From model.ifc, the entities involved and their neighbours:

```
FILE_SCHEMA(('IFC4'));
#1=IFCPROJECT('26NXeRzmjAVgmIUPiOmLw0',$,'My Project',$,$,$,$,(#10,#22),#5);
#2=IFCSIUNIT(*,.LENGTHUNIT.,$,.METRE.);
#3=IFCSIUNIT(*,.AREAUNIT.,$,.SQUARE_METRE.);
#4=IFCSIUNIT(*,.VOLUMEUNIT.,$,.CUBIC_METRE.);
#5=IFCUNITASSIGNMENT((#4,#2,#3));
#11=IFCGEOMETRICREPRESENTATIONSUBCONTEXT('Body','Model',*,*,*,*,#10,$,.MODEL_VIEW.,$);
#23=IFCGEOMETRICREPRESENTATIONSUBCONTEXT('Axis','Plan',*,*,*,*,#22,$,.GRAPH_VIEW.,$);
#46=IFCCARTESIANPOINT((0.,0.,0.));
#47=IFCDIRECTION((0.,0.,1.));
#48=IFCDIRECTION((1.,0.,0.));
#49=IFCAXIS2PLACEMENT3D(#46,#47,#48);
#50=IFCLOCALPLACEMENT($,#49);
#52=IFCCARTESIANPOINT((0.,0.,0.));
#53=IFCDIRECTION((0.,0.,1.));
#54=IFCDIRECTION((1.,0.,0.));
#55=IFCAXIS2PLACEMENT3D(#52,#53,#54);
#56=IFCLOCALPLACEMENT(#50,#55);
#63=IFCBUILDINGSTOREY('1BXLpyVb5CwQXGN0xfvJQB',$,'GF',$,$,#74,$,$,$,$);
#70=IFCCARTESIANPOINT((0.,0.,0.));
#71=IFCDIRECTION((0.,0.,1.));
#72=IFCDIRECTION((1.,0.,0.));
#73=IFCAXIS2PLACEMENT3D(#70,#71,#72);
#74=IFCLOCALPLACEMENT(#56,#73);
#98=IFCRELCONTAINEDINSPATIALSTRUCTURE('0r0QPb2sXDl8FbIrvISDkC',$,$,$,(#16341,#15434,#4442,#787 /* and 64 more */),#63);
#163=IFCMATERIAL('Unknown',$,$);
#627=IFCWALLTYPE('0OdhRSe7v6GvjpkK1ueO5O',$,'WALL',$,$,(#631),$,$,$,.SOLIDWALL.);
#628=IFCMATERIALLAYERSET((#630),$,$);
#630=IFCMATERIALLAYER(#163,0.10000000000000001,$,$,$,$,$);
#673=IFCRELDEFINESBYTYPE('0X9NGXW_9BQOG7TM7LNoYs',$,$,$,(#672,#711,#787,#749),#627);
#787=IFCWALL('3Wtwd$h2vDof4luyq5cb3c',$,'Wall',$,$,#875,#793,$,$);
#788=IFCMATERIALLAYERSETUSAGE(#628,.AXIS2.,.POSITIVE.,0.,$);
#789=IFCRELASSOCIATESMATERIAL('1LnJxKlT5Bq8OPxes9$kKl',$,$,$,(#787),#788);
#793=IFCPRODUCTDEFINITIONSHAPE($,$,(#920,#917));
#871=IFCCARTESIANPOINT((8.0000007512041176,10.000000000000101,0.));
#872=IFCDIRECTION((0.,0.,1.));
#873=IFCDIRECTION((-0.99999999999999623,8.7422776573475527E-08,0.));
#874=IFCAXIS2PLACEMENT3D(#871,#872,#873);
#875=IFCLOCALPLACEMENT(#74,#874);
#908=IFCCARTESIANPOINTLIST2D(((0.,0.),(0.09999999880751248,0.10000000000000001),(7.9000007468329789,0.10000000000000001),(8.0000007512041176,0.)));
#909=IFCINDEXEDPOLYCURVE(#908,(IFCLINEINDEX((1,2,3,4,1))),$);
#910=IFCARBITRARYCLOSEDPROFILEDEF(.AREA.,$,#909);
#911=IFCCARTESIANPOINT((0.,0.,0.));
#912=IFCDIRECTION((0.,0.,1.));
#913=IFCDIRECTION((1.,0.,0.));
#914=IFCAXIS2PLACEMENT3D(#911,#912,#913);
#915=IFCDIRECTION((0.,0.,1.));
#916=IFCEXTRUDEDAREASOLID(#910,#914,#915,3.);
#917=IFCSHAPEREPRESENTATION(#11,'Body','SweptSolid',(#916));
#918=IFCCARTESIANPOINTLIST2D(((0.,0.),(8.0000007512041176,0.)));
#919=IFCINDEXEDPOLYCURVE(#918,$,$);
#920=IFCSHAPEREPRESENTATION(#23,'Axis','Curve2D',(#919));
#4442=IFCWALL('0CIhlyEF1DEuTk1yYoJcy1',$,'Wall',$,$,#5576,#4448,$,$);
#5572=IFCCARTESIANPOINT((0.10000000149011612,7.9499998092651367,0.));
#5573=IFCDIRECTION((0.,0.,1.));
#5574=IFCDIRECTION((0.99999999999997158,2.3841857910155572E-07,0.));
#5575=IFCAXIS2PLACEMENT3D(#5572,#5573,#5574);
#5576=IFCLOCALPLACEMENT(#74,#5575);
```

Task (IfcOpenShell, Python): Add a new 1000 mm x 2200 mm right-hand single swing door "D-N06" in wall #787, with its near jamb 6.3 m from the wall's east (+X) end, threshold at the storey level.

```python
import numpy as np
import ifcopenshell
import ifcopenshell.api.feature
import ifcopenshell.api.geometry
import ifcopenshell.api.root
import ifcopenshell.api.spatial
import ifcopenshell.geom
import ifcopenshell.util.element
import ifcopenshell.util.placement
import ifcopenshell.util.representation
import ifcopenshell.util.shape
import ifcopenshell.util.unit

model = ifcopenshell.open("model.ifc")
unit_scale = ifcopenshell.util.unit.calculate_unit_scale(model)
settings = ifcopenshell.geom.settings()


def volume(element):
    """Net volume in cubic metres, openings subtracted."""
    shape = ifcopenshell.geom.create_shape(settings, element)
    return ifcopenshell.util.shape.get_volume(shape.geometry)


wall = model.by_guid("3Wtwd$h2vDof4luyq5cb3c")
storey = ifcopenshell.util.element.get_container(wall, ifc_class="IfcBuildingStorey")
context = ifcopenshell.util.representation.get_context(model, "Model", "Body", "MODEL_VIEW")
before = volume(wall)

width, height, from_end, sill = 1, 2.2, 6.3, 0.0  # metres

# The wall runs along its own X axis, and the end named is its -X end.
wall_shape = ifcopenshell.geom.create_shape(settings, wall)
x, y, z = ifcopenshell.util.shape.get_vertices(wall_shape.geometry).T
start = x.min() + from_end
face, thickness = float(y.min()), float(y.max() - y.min())
wall_matrix = ifcopenshell.util.placement.get_local_placement(wall.ObjectPlacement)
level = ifcopenshell.util.placement.get_local_placement(storey.ObjectPlacement)[2, 3]


def in_wall(x, y):
    """Placement at x, y metres in the wall's axes, at sill height."""
    matrix = wall_matrix.copy()
    matrix[:, 3] = wall_matrix @ np.array([x / unit_scale, y / unit_scale, 0.0, 1.0])
    matrix[2, 3] = level + sill / unit_scale
    return matrix


# Opening: a box that overshoots both wall faces by 50 mm.
opening = ifcopenshell.api.root.create_entity(model, ifc_class="IfcOpeningElement", predefined_type="OPENING")
box = ifcopenshell.api.geometry.add_wall_representation(
    model, context=context, length=width, height=height, thickness=thickness + 0.1
)
ifcopenshell.api.geometry.assign_representation(model, product=opening, representation=box)
ifcopenshell.api.geometry.edit_object_placement(model, product=opening, matrix=in_wall(start, face - 0.05), is_si=False)
ifcopenshell.api.feature.add_feature(model, feature=opening, element=wall)

door = ifcopenshell.api.root.create_entity(model, ifc_class="IfcDoor", name="D-N06", predefined_type="DOOR")
door.OverallWidth, door.OverallHeight = width / unit_scale, height / unit_scale
door.OperationType = "SINGLE_SWING_RIGHT"
body = ifcopenshell.api.geometry.add_door_representation(
    model,
    context=context,
    overall_width=door.OverallWidth,
    overall_height=door.OverallHeight,
    operation_type="SINGLE_SWING_RIGHT",
    lining_properties={"LiningDepth": thickness / unit_scale, "ThresholdDepth": thickness / unit_scale},
)
ifcopenshell.api.geometry.assign_representation(model, product=door, representation=body)
ifcopenshell.api.spatial.assign_container(model, products=[door], relating_structure=storey)
ifcopenshell.api.feature.add_filling(model, opening=opening, element=door)

# The lining spans the wall, so the door starts at the wall face.
ifcopenshell.api.geometry.edit_object_placement(model, product=door, matrix=in_wall(start, face), is_si=False)

after = volume(wall)

print(f"wall volume {before:.3f} -> {after:.3f} m3")

model.write("model_updated.ifc")
```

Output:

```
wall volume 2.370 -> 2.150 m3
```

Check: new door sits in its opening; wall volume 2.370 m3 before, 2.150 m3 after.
